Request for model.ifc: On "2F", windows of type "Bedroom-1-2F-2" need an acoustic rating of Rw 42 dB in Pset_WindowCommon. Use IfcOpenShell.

First a look at what the model holds.

```python
import ifcopenshell
import ifcopenshell.util.element

model = ifcopenshell.open("model.ifc")
print(model.schema)
storey = next(s for s in model.by_type("IfcBuildingStorey") if s.Name == "2F")
windows = [e for e in ifcopenshell.util.element.get_decomposition(storey) if e.is_a("IfcWindow")]
seen = {}
for e in windows:
    element_type = ifcopenshell.util.element.get_type(e)
    key = (element_type.Name if element_type != e and element_type else None, ifcopenshell.util.element.get_pset(e, "Pset_WindowCommon", "AcousticRating"))
    seen[key] = seen.get(key, 0) + 1
for (name, value), count in sorted(seen.items(), key=str):
    print(count, "x", name, "|", value)
```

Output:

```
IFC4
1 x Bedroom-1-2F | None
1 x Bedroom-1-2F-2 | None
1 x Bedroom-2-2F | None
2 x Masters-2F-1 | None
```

```python
import ifcopenshell
import ifcopenshell.api.pset
import ifcopenshell.util.element

model = ifcopenshell.open("model.ifc")

storey = next(s for s in model.by_type("IfcBuildingStorey") if s.Name == "2F")
windows = [e for e in ifcopenshell.util.element.get_decomposition(storey) if e.is_a("IfcWindow")]

count = 0
for e in windows:
    element_type = ifcopenshell.util.element.get_type(e)
    if element_type in (None, e) or element_type.Name != "Bedroom-1-2F-2":
        continue
    # add_pset returns the element's existing set when there is one.
    pset = ifcopenshell.api.pset.add_pset(model, product=e, name="Pset_WindowCommon")
    ifcopenshell.api.pset.edit_pset(model, pset=pset, properties={"AcousticRating": "Rw 42 dB"})
    count += 1

print(count, "windows updated")

model.write("model_rev.ifc")
```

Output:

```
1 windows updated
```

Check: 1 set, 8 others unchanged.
